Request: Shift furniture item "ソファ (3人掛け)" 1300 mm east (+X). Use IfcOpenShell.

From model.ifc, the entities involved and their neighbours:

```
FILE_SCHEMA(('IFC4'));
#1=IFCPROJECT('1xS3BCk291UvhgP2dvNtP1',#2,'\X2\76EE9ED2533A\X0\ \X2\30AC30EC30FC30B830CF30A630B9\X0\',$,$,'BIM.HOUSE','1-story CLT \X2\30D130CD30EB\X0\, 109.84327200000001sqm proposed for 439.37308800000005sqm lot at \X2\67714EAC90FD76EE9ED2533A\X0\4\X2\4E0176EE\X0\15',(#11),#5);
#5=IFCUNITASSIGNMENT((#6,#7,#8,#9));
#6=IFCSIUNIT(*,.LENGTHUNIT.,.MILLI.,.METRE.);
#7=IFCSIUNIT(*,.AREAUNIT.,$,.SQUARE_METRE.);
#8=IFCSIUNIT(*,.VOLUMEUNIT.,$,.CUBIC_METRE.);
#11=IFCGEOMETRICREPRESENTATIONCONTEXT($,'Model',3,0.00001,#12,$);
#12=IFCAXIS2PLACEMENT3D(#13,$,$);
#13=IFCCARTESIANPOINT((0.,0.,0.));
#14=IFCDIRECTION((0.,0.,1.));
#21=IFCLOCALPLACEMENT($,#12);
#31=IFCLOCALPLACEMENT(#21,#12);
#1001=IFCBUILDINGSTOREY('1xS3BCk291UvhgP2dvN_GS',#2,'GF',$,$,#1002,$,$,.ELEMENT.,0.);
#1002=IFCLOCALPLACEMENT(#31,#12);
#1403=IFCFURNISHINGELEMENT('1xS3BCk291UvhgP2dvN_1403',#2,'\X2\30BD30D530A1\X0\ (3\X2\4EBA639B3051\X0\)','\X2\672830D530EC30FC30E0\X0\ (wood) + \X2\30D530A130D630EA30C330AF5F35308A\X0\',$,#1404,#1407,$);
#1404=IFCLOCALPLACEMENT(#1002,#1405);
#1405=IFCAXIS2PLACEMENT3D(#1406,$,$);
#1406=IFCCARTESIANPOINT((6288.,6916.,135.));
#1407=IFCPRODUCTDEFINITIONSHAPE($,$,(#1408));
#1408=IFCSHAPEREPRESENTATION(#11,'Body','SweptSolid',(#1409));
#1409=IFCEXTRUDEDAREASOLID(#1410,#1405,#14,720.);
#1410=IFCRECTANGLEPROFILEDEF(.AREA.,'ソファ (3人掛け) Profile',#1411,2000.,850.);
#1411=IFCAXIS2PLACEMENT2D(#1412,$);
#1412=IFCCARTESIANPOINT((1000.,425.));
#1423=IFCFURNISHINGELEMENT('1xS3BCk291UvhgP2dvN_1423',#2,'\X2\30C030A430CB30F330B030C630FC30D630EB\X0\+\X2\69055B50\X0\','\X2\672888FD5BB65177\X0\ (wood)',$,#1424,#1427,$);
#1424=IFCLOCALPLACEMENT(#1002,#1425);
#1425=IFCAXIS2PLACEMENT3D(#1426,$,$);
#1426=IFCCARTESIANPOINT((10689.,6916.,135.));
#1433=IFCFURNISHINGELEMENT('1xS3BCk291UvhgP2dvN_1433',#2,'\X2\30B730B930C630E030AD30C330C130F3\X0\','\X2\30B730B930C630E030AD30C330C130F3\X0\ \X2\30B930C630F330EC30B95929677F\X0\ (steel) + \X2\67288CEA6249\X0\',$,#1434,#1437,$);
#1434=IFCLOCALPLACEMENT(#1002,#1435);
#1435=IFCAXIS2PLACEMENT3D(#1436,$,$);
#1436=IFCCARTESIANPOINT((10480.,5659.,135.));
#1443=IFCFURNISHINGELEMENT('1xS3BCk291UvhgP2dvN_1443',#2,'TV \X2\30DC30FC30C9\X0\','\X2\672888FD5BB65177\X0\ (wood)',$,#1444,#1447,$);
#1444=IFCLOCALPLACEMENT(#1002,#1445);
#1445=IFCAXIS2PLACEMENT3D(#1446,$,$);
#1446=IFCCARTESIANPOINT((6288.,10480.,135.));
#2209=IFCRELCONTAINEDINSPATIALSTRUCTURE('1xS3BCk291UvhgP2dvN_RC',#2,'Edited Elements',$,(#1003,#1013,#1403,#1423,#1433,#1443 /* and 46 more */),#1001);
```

```python
import ifcopenshell
import ifcopenshell.api.geometry
import ifcopenshell.util.placement
import ifcopenshell.util.unit

model = ifcopenshell.open("model.ifc")
unit_scale = ifcopenshell.util.unit.calculate_unit_scale(model)

item = model.by_id(1403)
matrix = ifcopenshell.util.placement.get_local_placement(item.ObjectPlacement)
matrix[0, 3] += 1.3 / unit_scale
ifcopenshell.api.geometry.edit_object_placement(model, product=item, matrix=matrix, is_si=False)

print(ifcopenshell.util.placement.get_local_placement(item.ObjectPlacement).round(3) + 0.0)

model.write("model_v2.ifc")
```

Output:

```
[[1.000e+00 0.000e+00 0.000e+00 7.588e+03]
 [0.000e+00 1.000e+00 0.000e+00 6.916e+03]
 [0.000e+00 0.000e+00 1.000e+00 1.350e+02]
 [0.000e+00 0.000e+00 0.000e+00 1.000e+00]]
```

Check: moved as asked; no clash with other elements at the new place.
